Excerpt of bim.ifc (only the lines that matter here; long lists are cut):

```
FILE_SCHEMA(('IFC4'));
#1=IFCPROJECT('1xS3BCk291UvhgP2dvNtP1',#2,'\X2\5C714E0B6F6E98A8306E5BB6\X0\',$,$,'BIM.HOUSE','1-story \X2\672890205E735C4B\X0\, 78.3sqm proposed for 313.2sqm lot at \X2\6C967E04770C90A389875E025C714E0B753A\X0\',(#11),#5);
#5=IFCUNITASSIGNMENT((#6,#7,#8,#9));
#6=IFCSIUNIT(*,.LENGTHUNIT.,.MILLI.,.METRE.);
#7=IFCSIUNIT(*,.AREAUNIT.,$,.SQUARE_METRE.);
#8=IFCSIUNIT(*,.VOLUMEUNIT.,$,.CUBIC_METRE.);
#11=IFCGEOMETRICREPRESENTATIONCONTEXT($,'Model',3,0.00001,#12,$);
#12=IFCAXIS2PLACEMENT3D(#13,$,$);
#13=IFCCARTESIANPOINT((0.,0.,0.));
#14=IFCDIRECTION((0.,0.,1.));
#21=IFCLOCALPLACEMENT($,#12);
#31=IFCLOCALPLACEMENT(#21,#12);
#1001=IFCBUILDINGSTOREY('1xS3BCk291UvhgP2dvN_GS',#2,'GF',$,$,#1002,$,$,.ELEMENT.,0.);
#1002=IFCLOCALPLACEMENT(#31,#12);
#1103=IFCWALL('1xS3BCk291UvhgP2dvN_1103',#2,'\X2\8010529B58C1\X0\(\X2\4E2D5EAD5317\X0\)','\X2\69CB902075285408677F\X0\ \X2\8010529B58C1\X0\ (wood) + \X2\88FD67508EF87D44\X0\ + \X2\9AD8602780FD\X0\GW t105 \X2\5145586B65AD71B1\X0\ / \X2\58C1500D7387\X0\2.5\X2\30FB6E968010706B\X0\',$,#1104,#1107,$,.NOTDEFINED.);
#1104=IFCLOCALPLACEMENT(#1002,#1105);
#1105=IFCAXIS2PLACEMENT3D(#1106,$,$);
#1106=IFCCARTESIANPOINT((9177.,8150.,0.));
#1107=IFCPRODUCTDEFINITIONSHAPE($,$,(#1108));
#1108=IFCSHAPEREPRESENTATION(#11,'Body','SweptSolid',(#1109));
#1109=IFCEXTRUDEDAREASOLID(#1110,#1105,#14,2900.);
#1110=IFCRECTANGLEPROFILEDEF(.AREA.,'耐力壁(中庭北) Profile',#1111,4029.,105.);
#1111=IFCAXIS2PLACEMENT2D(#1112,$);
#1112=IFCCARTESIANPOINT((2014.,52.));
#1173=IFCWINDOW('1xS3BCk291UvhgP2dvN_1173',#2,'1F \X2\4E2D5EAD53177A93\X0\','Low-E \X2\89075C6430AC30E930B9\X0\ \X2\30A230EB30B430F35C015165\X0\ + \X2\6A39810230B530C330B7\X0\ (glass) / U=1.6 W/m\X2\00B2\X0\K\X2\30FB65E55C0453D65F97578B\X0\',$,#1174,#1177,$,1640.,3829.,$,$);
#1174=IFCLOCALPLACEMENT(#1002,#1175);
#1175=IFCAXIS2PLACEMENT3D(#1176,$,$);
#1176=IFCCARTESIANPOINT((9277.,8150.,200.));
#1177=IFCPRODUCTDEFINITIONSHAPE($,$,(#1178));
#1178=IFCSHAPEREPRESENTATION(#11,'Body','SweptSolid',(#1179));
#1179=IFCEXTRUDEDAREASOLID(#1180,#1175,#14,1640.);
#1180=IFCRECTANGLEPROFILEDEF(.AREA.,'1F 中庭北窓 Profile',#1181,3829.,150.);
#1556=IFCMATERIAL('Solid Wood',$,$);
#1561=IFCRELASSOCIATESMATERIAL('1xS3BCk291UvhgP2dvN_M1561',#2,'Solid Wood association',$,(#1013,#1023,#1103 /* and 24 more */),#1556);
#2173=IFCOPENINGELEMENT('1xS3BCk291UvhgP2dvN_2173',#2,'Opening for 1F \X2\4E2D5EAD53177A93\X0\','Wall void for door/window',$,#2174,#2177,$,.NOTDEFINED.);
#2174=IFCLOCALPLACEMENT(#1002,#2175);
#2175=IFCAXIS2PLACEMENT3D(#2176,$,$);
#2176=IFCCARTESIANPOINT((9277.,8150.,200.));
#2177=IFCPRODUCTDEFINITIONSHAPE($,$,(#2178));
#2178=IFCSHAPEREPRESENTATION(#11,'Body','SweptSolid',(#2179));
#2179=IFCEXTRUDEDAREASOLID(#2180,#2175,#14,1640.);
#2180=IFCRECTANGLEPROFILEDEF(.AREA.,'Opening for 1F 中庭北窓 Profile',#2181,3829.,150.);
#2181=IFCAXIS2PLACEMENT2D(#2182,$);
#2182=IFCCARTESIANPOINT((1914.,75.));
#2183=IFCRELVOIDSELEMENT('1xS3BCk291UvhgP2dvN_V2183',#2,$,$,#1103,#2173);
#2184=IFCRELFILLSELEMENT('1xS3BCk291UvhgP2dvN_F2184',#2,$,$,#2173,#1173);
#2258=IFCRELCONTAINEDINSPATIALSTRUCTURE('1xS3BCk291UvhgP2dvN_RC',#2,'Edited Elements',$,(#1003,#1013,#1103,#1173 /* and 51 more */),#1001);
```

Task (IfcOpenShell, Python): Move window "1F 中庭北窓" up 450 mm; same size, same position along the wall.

```python
import numpy as np
import ifcopenshell
import ifcopenshell.api.geometry
import ifcopenshell.util.placement
import ifcopenshell.util.unit

model = ifcopenshell.open("bim.ifc")
unit_scale = ifcopenshell.util.unit.calculate_unit_scale(model)

window = model.by_guid("1xS3BCk291UvhgP2dvN_1173")
opening = window.FillsVoids[0].RelatingOpeningElement
dz = 0.45 / unit_scale

shift = np.array([0.0, 0.0, dz])
# The window is not placed relative to its opening, so move both.
for product in (opening, window):
    matrix = ifcopenshell.util.placement.get_local_placement(product.ObjectPlacement)
    matrix[:3, 3] += shift
    ifcopenshell.api.geometry.edit_object_placement(model, product=product, matrix=matrix, is_si=False)

print(f"moved by {dz * unit_scale:+.3f} m")

model.write("bim_updated.ifc")
```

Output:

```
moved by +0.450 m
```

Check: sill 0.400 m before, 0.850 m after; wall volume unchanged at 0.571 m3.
